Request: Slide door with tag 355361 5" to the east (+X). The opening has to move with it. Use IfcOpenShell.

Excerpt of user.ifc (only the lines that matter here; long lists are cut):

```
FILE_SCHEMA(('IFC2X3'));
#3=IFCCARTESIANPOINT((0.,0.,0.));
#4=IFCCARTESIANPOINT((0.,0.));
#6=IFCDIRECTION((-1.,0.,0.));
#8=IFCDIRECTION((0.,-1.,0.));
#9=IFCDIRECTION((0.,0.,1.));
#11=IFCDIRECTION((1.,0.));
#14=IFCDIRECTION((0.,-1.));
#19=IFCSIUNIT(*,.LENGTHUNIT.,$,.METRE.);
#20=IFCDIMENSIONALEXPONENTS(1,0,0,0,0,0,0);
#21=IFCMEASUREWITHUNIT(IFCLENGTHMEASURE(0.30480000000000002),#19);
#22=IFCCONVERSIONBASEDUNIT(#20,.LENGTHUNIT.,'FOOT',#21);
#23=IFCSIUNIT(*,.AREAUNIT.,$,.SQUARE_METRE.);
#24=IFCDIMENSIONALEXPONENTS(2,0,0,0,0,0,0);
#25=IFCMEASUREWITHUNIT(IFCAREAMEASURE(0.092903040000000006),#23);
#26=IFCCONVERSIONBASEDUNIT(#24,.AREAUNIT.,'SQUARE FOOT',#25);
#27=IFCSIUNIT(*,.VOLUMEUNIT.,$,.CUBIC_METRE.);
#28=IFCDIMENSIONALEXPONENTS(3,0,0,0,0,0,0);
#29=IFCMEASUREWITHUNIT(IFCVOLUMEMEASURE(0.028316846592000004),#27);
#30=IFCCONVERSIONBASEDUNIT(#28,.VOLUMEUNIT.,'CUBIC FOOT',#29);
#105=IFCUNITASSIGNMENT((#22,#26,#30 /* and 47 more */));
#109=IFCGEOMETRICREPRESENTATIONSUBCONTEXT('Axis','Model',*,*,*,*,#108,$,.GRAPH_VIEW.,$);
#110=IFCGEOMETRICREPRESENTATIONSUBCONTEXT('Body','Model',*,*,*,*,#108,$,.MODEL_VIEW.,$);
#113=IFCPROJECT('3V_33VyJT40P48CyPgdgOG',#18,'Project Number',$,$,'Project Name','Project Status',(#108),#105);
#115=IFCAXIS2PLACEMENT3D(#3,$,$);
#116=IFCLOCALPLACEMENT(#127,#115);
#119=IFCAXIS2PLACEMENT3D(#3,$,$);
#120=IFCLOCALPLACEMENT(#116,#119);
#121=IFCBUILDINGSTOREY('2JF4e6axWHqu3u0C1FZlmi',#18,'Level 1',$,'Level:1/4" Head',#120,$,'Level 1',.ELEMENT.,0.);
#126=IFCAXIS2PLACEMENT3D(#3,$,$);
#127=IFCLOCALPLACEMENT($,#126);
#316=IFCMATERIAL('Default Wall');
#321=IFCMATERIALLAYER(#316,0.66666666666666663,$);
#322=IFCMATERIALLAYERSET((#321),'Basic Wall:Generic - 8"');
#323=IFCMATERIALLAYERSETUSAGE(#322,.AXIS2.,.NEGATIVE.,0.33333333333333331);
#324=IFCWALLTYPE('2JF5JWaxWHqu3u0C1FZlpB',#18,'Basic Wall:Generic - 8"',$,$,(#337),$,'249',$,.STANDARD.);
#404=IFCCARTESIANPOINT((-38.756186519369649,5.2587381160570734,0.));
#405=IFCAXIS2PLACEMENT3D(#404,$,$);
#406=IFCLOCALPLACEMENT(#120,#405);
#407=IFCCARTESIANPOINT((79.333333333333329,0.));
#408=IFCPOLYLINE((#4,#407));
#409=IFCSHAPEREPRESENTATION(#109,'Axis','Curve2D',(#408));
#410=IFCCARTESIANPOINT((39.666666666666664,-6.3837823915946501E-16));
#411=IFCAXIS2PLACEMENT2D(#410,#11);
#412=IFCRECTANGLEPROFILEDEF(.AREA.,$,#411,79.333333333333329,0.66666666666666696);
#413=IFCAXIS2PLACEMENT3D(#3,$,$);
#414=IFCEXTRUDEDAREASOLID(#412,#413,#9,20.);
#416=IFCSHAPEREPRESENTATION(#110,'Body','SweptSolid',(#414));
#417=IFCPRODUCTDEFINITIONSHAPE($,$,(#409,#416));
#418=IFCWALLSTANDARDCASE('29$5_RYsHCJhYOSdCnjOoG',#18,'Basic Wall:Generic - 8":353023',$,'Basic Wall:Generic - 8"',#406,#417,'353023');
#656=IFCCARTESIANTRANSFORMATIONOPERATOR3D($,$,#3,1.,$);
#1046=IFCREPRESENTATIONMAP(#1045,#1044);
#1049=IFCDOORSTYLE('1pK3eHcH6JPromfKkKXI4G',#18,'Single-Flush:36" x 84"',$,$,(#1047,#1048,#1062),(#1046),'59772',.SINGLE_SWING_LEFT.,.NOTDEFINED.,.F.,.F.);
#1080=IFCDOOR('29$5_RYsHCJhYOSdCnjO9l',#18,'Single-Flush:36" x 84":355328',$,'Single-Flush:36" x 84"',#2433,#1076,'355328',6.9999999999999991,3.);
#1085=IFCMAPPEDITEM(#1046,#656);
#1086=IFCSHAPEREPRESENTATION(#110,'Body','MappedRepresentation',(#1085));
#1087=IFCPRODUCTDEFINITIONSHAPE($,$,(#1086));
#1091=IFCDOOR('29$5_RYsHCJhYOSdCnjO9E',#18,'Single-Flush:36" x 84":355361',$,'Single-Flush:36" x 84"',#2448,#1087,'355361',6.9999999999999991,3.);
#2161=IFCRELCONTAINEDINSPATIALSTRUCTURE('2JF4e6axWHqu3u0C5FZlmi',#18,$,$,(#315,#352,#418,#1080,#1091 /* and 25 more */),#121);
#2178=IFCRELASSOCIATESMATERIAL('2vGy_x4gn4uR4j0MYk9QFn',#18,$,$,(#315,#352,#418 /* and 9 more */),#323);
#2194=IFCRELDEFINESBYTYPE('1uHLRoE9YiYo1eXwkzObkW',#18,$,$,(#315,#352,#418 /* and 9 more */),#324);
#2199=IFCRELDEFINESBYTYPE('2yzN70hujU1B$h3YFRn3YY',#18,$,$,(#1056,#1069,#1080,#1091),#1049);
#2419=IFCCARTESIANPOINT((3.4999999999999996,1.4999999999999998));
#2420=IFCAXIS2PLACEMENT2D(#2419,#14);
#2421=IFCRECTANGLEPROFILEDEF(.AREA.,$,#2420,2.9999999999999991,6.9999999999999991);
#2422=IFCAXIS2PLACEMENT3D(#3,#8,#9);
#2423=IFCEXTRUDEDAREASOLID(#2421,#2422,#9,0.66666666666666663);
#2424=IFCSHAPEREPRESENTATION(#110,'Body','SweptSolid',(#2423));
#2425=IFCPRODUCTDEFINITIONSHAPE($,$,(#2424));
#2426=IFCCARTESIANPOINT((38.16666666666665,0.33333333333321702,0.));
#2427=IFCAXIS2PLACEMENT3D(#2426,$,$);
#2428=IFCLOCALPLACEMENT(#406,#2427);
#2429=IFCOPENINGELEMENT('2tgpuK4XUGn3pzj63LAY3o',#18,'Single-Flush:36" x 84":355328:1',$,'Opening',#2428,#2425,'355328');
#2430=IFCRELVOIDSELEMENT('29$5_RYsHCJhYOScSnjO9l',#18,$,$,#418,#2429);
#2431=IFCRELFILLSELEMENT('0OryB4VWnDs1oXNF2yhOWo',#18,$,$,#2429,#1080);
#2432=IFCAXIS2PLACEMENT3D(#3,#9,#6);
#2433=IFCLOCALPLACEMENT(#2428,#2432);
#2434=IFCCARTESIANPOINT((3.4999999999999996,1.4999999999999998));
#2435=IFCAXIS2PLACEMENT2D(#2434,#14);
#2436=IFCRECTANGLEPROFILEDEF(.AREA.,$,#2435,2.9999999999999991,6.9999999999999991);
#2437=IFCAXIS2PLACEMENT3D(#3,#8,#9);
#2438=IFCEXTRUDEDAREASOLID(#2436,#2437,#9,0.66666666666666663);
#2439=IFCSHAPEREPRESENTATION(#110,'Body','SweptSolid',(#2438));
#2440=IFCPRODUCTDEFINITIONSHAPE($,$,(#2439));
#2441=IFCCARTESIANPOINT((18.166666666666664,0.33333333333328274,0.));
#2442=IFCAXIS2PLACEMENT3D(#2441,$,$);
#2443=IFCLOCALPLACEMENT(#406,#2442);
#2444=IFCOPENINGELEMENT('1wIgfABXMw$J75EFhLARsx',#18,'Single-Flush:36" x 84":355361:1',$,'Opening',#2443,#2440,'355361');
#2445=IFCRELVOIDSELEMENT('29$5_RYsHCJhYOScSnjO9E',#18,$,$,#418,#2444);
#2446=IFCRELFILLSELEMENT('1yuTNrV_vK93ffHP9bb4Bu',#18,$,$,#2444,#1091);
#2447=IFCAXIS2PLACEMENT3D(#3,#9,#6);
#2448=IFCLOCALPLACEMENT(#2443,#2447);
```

```python
import ifcopenshell
import ifcopenshell.api.geometry
import ifcopenshell.util.placement
import ifcopenshell.util.unit

model = ifcopenshell.open("user.ifc")
unit_scale = ifcopenshell.util.unit.calculate_unit_scale(model)

door = model.by_id(1091)
opening = door.FillsVoids[0].RelatingOpeningElement
wall = opening.VoidsElements[0].RelatingBuildingElement

wall_matrix = ifcopenshell.util.placement.get_local_placement(wall.ObjectPlacement)
shift = wall_matrix[:3, 0] * 5 * 0.0254 / unit_scale
before = ifcopenshell.util.placement.get_local_placement(door.ObjectPlacement)[:3, 3].copy()

# The door is placed relative to its opening, so it follows when the opening moves.
matrix = ifcopenshell.util.placement.get_local_placement(opening.ObjectPlacement)
matrix[:3, 3] += shift
ifcopenshell.api.geometry.edit_object_placement(
    model, product=opening, matrix=matrix, is_si=False, should_transform_children=True
)

after = ifcopenshell.util.placement.get_local_placement(door.ObjectPlacement)[:3, 3]
print("door moved by", (after - before).round(3) + 0.0)

model.write("user_updated.ifc")
```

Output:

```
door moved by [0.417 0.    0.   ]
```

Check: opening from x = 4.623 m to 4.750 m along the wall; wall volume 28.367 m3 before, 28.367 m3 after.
